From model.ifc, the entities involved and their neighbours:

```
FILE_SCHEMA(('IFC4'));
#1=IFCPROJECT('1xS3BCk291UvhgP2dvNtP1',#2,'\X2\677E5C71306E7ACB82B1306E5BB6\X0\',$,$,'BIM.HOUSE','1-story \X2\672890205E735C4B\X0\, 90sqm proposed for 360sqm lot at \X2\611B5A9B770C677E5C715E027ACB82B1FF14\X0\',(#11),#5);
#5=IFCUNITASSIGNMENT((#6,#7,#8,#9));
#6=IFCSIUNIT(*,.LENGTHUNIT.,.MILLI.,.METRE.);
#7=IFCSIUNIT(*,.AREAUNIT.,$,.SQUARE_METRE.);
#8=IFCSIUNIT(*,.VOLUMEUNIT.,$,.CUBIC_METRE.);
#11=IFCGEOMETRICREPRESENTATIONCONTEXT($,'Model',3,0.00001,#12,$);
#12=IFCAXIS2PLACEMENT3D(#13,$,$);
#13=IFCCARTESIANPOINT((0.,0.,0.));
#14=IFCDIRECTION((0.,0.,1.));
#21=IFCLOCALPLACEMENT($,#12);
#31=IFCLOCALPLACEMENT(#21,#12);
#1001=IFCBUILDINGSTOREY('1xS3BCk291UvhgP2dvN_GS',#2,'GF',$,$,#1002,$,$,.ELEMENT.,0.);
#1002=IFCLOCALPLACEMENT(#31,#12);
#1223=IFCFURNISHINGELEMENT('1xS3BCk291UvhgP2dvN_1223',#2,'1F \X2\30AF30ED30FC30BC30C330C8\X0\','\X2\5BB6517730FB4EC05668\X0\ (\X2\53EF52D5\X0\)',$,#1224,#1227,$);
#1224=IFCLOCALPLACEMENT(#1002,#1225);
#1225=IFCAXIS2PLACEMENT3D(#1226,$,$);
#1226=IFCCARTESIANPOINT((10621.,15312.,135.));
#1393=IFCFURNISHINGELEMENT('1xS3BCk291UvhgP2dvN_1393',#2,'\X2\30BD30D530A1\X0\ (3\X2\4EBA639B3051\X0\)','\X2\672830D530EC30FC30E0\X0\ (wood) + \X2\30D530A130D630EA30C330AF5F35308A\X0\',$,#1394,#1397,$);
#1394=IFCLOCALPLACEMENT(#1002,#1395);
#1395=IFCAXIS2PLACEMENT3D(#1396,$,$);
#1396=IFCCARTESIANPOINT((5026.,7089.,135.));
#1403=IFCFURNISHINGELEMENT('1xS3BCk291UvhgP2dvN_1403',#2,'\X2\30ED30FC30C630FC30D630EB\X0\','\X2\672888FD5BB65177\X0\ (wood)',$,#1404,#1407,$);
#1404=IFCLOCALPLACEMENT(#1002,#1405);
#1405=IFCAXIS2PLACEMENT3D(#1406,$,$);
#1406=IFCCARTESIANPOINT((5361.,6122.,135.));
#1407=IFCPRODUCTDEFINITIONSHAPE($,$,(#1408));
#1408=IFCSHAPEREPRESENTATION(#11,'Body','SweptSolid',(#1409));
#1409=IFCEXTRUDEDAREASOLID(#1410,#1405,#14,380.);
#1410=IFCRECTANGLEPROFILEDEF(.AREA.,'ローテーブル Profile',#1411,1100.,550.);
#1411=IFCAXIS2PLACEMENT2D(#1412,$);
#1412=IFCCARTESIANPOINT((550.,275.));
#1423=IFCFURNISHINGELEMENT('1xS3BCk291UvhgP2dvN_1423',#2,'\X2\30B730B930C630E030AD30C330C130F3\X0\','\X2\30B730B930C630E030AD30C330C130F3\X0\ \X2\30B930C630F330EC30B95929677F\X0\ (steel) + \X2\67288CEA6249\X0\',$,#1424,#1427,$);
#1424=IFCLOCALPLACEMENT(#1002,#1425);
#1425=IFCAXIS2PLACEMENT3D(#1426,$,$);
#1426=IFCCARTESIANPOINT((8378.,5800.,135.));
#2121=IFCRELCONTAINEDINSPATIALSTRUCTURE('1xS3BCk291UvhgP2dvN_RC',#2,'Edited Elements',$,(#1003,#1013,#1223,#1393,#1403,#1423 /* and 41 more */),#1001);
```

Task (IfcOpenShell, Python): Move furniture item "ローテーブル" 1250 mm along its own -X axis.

```python
import ifcopenshell
import ifcopenshell.api.geometry
import ifcopenshell.util.placement
import ifcopenshell.util.unit

model = ifcopenshell.open("model.ifc")
unit_scale = ifcopenshell.util.unit.calculate_unit_scale(model)

item = model.by_guid("1xS3BCk291UvhgP2dvN_1403")
matrix = ifcopenshell.util.placement.get_local_placement(item.ObjectPlacement)
matrix[:3, 3] -= matrix[:3, 0] * 1.25 / unit_scale
ifcopenshell.api.geometry.edit_object_placement(model, product=item, matrix=matrix, is_si=False)

print(ifcopenshell.util.placement.get_local_placement(item.ObjectPlacement).round(3) + 0.0)

model.write("model_updated.ifc")
```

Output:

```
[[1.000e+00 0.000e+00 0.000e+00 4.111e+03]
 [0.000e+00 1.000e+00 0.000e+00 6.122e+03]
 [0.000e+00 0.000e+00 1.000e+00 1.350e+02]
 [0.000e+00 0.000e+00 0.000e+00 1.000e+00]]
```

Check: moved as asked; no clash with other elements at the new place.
